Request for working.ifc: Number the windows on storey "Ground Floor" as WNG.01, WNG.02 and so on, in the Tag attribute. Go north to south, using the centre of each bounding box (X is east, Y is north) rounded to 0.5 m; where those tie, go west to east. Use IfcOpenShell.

First a look at what the model holds.

```python
import ifcopenshell
import ifcopenshell.util.element
import ifcopenshell.util.placement

model = ifcopenshell.open("working.ifc")
print(model.schema)
storey = next(s for s in model.by_type("IfcBuildingStorey") if s.Name == "Ground Floor")
windows = [e for e in ifcopenshell.util.element.get_decomposition(storey) if e.is_a("IfcWindow")]
for e in sorted(windows, key=lambda e: e.id()):
    origin = ifcopenshell.util.placement.get_local_placement(e.ObjectPlacement)[:3, 3]
    print(e.id(), e.Tag, e.Name, origin.round(2) + 0.0, sep=" | ")
```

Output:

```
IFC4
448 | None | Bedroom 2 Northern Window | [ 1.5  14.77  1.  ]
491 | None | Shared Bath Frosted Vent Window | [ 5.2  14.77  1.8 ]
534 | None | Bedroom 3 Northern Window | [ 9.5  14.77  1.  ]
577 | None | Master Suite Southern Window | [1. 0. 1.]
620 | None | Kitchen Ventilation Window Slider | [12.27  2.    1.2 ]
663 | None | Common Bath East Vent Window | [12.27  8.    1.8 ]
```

```python
import ifcopenshell
import ifcopenshell.geom
import ifcopenshell.util.element
import ifcopenshell.util.shape

model = ifcopenshell.open("working.ifc")
settings = ifcopenshell.geom.settings()
settings.set("use-world-coords", True)


def centre(element):
    shape = ifcopenshell.geom.create_shape(settings, element)
    return ifcopenshell.util.shape.get_bbox_centroid(shape.geometry)


storey = next(s for s in model.by_type("IfcBuildingStorey") if s.Name == "Ground Floor")
windows = [e for e in ifcopenshell.util.element.get_decomposition(storey) if e.is_a("IfcWindow")]

# Insertion points can sit at a corner or the storey origin, so sort by the geometry (in metres).
centres = {e: centre(e) for e in windows}
windows.sort(key=lambda e: (-round(centres[e][1] / 0.5), centres[e][0]))

for i, e in enumerate(windows, start=1):
    number = f"WNG.{i:02d}"
    e.Tag = number
    print(e.id(), number)

model.write("working_edited.ifc")
```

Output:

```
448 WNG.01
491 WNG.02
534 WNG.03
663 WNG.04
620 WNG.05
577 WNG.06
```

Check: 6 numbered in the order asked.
